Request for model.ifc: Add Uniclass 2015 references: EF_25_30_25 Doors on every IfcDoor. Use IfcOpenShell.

First a look at what the model holds.

```python
import ifcopenshell

model = ifcopenshell.open("model.ifc")
print(model.schema)
print("classifications:", [c.Name for c in model.by_type("IfcClassification")])
for ifc_class in ("IfcDoor", "IfcRoof", "IfcStair", "IfcWall", "IfcWindow"):
    print(ifc_class, len(model.by_type(ifc_class)))
```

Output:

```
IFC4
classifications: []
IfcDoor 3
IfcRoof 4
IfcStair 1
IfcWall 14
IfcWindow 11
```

```python
import ifcopenshell
import ifcopenshell.api.classification

model = ifcopenshell.open("model.ifc")

system = ifcopenshell.api.classification.add_classification(model, classification="Uniclass 2015")

codes = {
    "IfcDoor": ("EF_25_30_25", "Doors"),
}
for ifc_class, (code, name) in codes.items():
    products = model.by_type(ifc_class)
    ifcopenshell.api.classification.add_reference(
        model, products=products, classification=system, identification=code, name=name
    )
    print(code, len(products))

model.write("model_updated.ifc")
```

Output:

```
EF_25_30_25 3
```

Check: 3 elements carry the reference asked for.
